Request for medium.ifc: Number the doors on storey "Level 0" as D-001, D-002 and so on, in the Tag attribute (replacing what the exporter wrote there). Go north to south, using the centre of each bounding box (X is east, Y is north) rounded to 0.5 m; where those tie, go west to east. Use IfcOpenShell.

First a look at what the model holds.

```python
import ifcopenshell
import ifcopenshell.util.element
import ifcopenshell.util.placement

model = ifcopenshell.open("medium.ifc")
print(model.schema)
storey = next(s for s in model.by_type("IfcBuildingStorey") if s.Name == "Level 0")
doors = [e for e in ifcopenshell.util.element.get_decomposition(storey) if e.is_a("IfcDoor")]
for e in sorted(doors, key=lambda e: e.id()):
    origin = ifcopenshell.util.placement.get_local_placement(e.ObjectPlacement)[:3, 3]
    print(e.id(), e.Tag, e.Name, origin.round(2) + 0.0, sep=" | ")
```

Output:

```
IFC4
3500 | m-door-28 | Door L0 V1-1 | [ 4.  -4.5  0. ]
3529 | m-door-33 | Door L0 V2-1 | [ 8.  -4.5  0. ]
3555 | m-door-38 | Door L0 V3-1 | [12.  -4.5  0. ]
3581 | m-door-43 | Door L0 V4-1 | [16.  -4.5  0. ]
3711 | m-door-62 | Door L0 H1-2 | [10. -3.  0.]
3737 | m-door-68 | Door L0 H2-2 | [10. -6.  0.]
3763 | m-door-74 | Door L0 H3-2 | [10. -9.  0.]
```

```python
import ifcopenshell
import ifcopenshell.geom
import ifcopenshell.util.element
import ifcopenshell.util.shape

model = ifcopenshell.open("medium.ifc")
settings = ifcopenshell.geom.settings()
settings.set("use-world-coords", True)


def centre(element):
    shape = ifcopenshell.geom.create_shape(settings, element)
    return ifcopenshell.util.shape.get_bbox_centroid(shape.geometry)


storey = next(s for s in model.by_type("IfcBuildingStorey") if s.Name == "Level 0")
doors = [e for e in ifcopenshell.util.element.get_decomposition(storey) if e.is_a("IfcDoor")]

# Insertion points can sit at a corner or the storey origin, so sort by the geometry (in metres).
centres = {e: centre(e) for e in doors}
doors.sort(key=lambda e: (-round(centres[e][1] / 0.5), centres[e][0]))

for i, e in enumerate(doors, start=1):
    number = f"D-0{i:02d}"
    e.Tag = number
    print(e.id(), number)

model.write("medium_edited.ifc")
```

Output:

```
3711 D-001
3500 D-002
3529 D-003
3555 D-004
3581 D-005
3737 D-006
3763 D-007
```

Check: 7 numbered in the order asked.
